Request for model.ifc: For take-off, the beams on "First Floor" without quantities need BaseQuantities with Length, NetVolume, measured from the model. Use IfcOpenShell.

First a look at what the model holds.

```python
import ifcopenshell
import ifcopenshell.util.element
import ifcopenshell.util.unit

model = ifcopenshell.open("model.ifc")
print(model.schema)
for unit_type in ("LENGTHUNIT", "AREAUNIT", "VOLUMEUNIT"):
    print(unit_type, ifcopenshell.util.unit.calculate_unit_scale(model, unit_type))
storey = next(s for s in model.by_type("IfcBuildingStorey") if s.Name == "First Floor")
beams = [e for e in ifcopenshell.util.element.get_decomposition(storey) if e.is_a("IfcBeam")]
for e in sorted(beams, key=lambda e: e.id()):
    print(e.id(), e.is_a(), e.Name, list(ifcopenshell.util.element.get_psets(e, qtos_only=True)), sep=" | ")
```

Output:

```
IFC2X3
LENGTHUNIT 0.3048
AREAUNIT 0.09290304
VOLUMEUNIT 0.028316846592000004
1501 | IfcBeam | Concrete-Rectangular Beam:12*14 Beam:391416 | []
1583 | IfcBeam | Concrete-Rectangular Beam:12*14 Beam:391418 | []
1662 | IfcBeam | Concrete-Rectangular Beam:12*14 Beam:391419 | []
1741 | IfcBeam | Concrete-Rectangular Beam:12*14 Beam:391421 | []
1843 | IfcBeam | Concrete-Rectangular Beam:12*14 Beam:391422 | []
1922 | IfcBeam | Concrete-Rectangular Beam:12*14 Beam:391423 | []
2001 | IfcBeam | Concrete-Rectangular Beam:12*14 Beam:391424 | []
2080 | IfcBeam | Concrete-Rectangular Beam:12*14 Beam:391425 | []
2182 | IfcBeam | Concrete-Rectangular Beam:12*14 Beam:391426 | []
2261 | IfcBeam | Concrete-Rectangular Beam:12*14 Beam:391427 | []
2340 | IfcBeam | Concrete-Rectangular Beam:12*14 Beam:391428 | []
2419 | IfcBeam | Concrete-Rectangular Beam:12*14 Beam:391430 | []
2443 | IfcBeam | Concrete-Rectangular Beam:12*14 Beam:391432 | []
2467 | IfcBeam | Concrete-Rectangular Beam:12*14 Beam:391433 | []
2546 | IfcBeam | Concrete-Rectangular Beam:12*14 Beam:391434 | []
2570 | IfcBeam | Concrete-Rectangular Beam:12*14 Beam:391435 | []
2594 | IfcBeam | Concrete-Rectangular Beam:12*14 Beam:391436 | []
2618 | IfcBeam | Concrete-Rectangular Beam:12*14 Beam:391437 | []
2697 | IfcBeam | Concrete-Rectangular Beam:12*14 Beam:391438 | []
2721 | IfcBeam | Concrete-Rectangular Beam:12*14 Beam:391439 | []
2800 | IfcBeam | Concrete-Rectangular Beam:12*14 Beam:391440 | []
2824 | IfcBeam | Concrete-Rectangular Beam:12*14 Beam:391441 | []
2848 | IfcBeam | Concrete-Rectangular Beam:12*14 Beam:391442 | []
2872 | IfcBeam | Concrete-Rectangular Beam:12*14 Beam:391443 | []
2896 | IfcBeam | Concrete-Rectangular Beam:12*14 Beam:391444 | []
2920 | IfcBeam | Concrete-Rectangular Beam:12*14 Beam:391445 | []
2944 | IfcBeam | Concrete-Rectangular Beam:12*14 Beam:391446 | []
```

```python
import ifcopenshell
import ifcopenshell.api.pset
import ifcopenshell.geom
import ifcopenshell.util.element
import ifcopenshell.util.shape
import ifcopenshell.util.unit

model = ifcopenshell.open("model.ifc")
unit_scale = ifcopenshell.util.unit.calculate_unit_scale(model)
volume_scale = ifcopenshell.util.unit.calculate_unit_scale(model, "VOLUMEUNIT")
settings = ifcopenshell.geom.settings()

storey = next(s for s in model.by_type("IfcBuildingStorey") if s.Name == "First Floor")
beams = [e for e in ifcopenshell.util.element.get_decomposition(storey) if e.is_a("IfcBeam")]

for e in sorted(beams, key=lambda e: e.id()):
    if ifcopenshell.util.element.get_psets(e, qtos_only=True, should_inherit=False):
        continue
    # Geometry comes back in metres, in the element's own axes.
    shape = ifcopenshell.geom.create_shape(settings, e)
    values = {
        "Length": ifcopenshell.util.shape.get_max_xyz(shape.geometry) / unit_scale,
        "NetVolume": ifcopenshell.util.shape.get_volume(shape.geometry) / volume_scale,
    }
    qto = ifcopenshell.api.pset.add_qto(model, product=e, name="BaseQuantities")
    ifcopenshell.api.pset.edit_qto(model, qto=qto, properties=values)
    print(e.id(), {k: round(v, 3) for k, v in values.items()})

model.write("model_rev.ifc")
```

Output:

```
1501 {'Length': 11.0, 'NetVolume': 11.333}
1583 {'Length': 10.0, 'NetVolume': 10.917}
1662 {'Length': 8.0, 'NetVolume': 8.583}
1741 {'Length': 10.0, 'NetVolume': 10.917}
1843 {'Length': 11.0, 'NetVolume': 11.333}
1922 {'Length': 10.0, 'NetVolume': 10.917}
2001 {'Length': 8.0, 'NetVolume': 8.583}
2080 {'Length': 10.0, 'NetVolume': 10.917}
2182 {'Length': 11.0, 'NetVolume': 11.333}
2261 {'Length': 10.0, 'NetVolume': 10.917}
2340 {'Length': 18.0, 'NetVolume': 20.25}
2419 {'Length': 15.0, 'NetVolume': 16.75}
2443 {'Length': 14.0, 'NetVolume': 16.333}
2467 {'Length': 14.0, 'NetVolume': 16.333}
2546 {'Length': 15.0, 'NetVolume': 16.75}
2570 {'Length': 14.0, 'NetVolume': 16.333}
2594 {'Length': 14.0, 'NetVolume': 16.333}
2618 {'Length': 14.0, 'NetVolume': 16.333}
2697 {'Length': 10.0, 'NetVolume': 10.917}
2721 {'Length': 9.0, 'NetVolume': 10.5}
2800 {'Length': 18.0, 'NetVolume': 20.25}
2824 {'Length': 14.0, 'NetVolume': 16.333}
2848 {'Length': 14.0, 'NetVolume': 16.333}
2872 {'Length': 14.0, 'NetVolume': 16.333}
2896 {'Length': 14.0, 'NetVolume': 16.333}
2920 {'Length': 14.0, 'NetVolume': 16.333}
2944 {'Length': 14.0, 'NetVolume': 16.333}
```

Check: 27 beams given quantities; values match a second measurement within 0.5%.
